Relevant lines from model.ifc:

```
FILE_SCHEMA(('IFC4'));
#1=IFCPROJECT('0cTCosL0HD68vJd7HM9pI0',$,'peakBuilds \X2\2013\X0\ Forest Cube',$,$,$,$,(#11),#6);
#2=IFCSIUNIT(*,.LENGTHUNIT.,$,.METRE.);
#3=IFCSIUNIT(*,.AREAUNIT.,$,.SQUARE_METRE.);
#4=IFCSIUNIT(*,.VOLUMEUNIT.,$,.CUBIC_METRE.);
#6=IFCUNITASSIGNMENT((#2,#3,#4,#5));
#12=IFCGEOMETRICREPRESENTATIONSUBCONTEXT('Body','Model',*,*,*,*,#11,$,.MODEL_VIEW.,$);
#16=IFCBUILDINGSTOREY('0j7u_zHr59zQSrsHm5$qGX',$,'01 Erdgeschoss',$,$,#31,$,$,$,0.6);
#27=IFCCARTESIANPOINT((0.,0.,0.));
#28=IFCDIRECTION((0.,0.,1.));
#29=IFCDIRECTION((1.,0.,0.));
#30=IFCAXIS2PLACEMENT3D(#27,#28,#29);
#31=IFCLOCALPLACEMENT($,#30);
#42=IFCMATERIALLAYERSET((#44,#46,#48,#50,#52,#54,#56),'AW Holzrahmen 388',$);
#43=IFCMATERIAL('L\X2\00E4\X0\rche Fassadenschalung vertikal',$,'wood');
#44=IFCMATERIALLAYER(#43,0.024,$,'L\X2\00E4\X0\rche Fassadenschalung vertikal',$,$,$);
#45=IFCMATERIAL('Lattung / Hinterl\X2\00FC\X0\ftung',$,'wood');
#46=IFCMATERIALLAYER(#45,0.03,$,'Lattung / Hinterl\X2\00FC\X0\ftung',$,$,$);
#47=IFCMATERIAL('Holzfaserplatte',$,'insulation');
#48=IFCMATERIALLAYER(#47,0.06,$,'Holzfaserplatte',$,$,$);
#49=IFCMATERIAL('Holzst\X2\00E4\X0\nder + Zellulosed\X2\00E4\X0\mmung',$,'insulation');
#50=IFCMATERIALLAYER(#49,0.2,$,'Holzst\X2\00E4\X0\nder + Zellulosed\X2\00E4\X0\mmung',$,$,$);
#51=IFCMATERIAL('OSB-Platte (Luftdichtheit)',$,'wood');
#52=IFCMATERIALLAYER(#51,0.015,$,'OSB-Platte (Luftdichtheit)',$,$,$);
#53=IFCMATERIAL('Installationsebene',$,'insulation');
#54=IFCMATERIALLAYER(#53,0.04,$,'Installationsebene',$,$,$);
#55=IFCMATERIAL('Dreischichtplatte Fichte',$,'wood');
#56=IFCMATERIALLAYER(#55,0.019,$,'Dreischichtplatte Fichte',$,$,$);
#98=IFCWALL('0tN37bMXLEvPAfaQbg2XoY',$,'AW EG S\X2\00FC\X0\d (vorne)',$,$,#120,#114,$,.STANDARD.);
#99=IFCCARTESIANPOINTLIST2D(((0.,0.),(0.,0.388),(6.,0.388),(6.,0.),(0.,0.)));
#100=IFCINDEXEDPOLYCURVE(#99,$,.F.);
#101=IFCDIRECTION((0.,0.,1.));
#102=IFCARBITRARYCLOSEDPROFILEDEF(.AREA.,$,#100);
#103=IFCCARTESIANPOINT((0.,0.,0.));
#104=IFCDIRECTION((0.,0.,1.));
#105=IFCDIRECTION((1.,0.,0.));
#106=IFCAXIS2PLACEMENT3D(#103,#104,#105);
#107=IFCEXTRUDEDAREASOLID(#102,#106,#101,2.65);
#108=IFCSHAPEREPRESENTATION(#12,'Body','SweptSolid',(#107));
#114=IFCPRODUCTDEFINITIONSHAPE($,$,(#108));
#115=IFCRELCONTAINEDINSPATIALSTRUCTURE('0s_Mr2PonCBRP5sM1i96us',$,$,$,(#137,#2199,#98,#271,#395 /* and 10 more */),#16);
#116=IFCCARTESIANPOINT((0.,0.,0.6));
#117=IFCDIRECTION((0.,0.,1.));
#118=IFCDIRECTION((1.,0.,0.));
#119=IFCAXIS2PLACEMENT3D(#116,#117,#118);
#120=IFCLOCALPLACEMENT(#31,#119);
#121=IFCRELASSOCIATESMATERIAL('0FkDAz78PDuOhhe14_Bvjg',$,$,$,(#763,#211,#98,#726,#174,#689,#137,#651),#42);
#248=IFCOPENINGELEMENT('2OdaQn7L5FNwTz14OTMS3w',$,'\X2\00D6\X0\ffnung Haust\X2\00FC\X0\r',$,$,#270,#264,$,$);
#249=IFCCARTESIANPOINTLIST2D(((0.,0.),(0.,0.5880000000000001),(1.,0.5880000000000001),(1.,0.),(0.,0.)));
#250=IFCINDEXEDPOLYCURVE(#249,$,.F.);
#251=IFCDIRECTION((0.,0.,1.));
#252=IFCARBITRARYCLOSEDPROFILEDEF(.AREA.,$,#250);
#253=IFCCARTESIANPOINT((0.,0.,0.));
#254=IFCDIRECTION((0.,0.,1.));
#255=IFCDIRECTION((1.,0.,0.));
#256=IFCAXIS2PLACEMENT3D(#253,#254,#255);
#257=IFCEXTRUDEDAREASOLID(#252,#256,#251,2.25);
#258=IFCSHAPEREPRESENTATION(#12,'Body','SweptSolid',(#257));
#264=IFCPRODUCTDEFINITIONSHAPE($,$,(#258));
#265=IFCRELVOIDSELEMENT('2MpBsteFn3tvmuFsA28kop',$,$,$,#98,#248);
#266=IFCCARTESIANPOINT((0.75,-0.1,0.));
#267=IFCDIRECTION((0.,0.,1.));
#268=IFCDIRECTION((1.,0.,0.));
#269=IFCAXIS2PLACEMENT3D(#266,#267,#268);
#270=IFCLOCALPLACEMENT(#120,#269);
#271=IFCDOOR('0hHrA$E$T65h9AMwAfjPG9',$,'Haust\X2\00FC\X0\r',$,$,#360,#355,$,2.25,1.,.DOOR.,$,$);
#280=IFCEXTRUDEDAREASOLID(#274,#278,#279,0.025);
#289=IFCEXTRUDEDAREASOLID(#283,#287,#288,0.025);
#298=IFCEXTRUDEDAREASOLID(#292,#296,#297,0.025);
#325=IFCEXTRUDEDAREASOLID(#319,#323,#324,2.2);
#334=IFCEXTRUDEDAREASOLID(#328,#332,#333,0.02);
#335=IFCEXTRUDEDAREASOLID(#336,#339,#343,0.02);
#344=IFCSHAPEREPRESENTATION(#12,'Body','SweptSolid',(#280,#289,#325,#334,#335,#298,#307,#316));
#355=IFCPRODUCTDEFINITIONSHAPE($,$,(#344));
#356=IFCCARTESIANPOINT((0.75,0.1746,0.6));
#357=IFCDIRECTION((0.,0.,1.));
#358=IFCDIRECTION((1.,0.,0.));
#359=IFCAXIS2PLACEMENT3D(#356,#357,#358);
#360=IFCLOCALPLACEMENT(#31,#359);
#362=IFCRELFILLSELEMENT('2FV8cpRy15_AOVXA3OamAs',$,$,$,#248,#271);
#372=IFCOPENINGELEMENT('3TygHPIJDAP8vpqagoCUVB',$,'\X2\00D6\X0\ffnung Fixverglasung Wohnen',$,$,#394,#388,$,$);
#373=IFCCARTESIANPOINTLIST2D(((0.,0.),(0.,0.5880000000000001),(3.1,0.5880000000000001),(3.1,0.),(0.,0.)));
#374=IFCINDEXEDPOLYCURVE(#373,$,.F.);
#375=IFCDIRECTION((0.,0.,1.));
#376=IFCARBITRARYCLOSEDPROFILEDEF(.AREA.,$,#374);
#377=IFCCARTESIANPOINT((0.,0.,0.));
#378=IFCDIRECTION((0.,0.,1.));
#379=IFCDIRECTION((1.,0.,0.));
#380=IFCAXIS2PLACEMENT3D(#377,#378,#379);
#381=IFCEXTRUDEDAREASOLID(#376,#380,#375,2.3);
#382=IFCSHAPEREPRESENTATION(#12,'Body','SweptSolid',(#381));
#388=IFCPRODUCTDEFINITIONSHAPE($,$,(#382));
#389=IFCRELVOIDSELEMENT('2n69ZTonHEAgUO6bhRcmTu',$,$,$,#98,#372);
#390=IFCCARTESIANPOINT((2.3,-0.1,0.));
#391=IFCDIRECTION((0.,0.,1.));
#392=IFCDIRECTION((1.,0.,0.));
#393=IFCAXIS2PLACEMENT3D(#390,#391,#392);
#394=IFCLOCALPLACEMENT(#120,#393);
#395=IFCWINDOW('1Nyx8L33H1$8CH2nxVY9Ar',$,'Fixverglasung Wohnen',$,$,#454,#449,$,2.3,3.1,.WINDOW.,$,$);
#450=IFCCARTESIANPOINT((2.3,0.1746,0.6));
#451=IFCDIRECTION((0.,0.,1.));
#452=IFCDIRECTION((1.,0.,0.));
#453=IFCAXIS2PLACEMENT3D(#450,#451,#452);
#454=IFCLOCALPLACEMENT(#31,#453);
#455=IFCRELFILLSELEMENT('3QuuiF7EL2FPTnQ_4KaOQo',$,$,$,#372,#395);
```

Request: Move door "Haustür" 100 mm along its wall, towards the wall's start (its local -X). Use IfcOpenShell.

```python
import ifcopenshell
import ifcopenshell.api.geometry
import ifcopenshell.util.placement
import ifcopenshell.util.unit

model = ifcopenshell.open("model.ifc")
unit_scale = ifcopenshell.util.unit.calculate_unit_scale(model)

door = model.by_id(271)
opening = door.FillsVoids[0].RelatingOpeningElement
wall = opening.VoidsElements[0].RelatingBuildingElement

wall_matrix = ifcopenshell.util.placement.get_local_placement(wall.ObjectPlacement)
shift = wall_matrix[:3, 0] * -0.1 / unit_scale
before = ifcopenshell.util.placement.get_local_placement(door.ObjectPlacement)[:3, 3].copy()

# The door is not placed relative to its opening, so move both.
for product in (opening, door):
    matrix = ifcopenshell.util.placement.get_local_placement(product.ObjectPlacement)
    matrix[:3, 3] += shift
    ifcopenshell.api.geometry.edit_object_placement(model, product=product, matrix=matrix, is_si=False)

after = ifcopenshell.util.placement.get_local_placement(door.ObjectPlacement)[:3, 3]
print("door moved by", (after - before).round(3) + 0.0)

model.write("model_updated.ifc")
```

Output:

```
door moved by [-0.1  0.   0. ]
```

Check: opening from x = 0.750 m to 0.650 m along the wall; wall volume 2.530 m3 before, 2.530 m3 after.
